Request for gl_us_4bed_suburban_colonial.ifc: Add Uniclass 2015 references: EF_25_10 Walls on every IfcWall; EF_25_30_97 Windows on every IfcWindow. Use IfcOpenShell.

First a look at what the model holds.

```python
import ifcopenshell

model = ifcopenshell.open("gl_us_4bed_suburban_colonial.ifc")
print(model.schema)
print("classifications:", [c.Name for c in model.by_type("IfcClassification")])
for ifc_class in ("IfcDoor", "IfcRoof", "IfcStair", "IfcWall", "IfcWindow"):
    print(ifc_class, len(model.by_type(ifc_class)))
```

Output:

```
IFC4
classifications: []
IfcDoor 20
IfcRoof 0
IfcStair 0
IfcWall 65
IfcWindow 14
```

```python
import ifcopenshell
import ifcopenshell.api.classification

model = ifcopenshell.open("gl_us_4bed_suburban_colonial.ifc")

system = ifcopenshell.api.classification.add_classification(model, classification="Uniclass 2015")

codes = {
    "IfcWall": ("EF_25_10", "Walls"),
    "IfcWindow": ("EF_25_30_97", "Windows"),
}
for ifc_class, (code, name) in codes.items():
    products = model.by_type(ifc_class)
    ifcopenshell.api.classification.add_reference(
        model, products=products, classification=system, identification=code, name=name
    )
    print(code, len(products))

model.write("gl_us_4bed_suburban_colonial_v2.ifc")
```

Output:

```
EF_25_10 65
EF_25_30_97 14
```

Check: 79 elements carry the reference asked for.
